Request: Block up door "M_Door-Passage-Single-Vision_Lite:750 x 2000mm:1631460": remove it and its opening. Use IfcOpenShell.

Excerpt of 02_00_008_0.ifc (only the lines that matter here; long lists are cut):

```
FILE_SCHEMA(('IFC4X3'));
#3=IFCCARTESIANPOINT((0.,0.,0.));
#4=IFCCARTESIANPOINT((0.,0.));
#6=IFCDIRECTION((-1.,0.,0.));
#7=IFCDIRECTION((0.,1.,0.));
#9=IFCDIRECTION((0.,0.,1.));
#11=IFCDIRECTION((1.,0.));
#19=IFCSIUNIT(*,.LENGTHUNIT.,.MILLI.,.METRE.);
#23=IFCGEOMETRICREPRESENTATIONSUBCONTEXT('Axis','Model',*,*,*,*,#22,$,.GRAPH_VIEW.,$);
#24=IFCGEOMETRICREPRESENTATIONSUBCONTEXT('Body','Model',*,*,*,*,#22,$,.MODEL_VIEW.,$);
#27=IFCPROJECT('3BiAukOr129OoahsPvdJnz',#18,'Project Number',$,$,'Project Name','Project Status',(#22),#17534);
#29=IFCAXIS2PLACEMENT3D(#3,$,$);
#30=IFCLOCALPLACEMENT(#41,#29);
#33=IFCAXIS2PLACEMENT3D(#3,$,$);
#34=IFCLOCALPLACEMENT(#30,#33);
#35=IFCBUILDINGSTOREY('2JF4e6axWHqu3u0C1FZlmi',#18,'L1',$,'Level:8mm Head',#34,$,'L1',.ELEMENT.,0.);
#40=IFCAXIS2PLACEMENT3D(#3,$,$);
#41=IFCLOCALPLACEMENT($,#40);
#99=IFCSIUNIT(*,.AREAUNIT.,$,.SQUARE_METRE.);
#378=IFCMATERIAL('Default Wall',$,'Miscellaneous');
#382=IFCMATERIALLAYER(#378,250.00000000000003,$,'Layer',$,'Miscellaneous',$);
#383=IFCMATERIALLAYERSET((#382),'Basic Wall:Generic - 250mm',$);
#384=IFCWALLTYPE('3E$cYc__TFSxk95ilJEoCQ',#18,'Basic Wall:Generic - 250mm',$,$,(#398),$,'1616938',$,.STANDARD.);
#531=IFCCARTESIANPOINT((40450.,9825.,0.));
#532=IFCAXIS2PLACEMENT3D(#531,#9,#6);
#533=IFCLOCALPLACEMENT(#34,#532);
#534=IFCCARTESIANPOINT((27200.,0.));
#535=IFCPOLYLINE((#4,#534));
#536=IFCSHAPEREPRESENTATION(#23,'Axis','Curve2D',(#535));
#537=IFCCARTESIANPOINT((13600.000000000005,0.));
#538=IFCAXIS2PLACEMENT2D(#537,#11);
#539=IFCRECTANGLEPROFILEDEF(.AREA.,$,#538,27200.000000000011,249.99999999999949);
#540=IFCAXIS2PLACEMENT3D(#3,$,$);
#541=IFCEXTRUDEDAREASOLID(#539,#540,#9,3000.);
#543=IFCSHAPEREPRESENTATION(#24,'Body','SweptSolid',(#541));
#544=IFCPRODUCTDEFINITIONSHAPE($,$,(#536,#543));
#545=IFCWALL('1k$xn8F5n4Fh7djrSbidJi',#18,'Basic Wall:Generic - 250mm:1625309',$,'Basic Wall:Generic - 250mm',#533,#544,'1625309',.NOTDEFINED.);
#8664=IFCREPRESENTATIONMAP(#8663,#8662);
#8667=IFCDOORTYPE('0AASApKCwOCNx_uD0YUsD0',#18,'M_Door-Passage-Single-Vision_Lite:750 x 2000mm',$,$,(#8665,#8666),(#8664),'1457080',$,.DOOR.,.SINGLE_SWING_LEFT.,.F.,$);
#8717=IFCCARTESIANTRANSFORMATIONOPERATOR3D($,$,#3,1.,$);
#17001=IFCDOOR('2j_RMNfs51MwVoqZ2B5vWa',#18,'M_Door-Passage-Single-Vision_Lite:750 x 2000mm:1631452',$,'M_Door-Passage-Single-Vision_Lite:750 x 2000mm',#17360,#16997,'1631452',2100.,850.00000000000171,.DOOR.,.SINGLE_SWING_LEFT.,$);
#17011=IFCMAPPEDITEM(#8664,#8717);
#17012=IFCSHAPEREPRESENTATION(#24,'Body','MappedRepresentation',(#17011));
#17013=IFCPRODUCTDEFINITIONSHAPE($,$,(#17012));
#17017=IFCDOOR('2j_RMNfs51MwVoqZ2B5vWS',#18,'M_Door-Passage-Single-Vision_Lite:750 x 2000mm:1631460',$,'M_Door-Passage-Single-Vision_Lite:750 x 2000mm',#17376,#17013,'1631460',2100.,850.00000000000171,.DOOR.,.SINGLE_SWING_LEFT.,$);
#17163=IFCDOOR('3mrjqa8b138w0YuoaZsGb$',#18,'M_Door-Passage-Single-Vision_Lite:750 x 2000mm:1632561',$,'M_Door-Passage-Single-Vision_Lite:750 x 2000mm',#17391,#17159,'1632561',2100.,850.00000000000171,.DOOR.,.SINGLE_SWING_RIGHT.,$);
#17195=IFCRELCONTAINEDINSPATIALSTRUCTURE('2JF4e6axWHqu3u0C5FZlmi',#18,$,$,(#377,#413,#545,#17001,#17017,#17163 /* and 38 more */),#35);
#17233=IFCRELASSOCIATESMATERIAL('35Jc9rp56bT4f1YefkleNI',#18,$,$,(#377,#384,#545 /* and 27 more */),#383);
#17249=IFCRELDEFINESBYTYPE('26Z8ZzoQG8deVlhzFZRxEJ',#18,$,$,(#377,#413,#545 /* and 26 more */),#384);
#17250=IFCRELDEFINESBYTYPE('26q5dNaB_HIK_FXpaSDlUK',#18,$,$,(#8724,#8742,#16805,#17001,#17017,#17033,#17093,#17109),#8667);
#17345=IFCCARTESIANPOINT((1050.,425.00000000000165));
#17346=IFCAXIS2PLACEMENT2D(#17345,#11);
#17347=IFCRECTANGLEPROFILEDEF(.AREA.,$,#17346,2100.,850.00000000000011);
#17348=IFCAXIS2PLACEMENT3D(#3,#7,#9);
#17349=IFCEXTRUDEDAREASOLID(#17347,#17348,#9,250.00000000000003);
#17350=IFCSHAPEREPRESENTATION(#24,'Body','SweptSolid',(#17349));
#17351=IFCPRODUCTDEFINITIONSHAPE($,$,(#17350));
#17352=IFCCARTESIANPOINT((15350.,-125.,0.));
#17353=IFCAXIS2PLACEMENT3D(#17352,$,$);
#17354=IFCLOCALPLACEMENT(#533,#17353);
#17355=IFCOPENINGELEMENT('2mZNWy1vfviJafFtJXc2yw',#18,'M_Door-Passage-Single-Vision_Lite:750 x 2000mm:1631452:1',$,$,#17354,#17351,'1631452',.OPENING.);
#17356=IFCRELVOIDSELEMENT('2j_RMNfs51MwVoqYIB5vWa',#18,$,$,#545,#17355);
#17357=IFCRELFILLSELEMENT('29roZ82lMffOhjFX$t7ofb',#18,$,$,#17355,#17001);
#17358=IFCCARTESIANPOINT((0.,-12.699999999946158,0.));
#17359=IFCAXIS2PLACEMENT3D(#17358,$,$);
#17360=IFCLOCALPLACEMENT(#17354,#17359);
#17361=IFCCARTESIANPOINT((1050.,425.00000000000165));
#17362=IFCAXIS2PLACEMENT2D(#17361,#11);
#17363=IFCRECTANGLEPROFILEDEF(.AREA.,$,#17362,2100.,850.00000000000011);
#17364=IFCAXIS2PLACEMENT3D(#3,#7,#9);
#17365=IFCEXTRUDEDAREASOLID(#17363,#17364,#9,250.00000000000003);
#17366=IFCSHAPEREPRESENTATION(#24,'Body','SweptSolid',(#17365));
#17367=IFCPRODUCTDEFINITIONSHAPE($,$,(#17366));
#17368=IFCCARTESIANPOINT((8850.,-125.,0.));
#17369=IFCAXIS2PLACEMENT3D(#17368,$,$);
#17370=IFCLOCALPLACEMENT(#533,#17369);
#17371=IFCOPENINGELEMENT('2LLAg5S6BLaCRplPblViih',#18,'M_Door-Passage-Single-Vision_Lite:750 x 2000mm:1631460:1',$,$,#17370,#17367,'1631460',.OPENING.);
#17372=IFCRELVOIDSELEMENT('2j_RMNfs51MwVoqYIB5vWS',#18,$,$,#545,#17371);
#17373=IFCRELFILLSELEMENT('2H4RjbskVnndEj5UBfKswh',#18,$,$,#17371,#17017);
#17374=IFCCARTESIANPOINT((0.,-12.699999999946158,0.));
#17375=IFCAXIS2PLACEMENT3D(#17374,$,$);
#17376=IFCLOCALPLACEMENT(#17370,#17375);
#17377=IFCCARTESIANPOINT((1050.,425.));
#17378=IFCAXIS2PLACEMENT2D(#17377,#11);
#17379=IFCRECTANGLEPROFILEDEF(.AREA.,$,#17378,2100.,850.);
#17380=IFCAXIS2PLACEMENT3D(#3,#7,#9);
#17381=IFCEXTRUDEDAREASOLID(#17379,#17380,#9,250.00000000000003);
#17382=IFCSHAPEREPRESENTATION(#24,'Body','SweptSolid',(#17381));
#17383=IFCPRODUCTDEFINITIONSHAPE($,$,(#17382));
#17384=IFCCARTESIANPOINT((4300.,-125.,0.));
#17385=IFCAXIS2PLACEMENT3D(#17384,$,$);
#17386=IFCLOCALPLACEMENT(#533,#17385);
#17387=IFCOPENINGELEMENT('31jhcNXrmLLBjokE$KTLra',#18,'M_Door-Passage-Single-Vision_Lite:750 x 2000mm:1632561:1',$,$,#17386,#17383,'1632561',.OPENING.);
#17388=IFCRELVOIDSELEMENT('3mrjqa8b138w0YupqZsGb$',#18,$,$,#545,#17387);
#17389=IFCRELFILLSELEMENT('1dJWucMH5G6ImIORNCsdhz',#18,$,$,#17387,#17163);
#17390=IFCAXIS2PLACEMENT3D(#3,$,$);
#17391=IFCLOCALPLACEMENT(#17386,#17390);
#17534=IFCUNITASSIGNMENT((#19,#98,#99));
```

```python
import ifcopenshell
import ifcopenshell.api.feature
import ifcopenshell.api.root
import ifcopenshell.geom
import ifcopenshell.util.shape

model = ifcopenshell.open("02_00_008_0.ifc")
settings = ifcopenshell.geom.settings()


def volume(element):
    """Net volume in cubic metres, openings subtracted."""
    shape = ifcopenshell.geom.create_shape(settings, element)
    return ifcopenshell.util.shape.get_volume(shape.geometry)


door = model.by_guid("2j_RMNfs51MwVoqZ2B5vWS")
opening = door.FillsVoids[0].RelatingOpeningElement
wall = opening.VoidsElements[0].RelatingBuildingElement
before = volume(wall)

ifcopenshell.api.root.remove_product(model, product=door)
ifcopenshell.api.feature.remove_feature(model, feature=opening)

after = volume(wall)

print(f"wall volume {before:.3f} -> {after:.3f} m3")

model.write("02_00_008_0_edited.ifc")
```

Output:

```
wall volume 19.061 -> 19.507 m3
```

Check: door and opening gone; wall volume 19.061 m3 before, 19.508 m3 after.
